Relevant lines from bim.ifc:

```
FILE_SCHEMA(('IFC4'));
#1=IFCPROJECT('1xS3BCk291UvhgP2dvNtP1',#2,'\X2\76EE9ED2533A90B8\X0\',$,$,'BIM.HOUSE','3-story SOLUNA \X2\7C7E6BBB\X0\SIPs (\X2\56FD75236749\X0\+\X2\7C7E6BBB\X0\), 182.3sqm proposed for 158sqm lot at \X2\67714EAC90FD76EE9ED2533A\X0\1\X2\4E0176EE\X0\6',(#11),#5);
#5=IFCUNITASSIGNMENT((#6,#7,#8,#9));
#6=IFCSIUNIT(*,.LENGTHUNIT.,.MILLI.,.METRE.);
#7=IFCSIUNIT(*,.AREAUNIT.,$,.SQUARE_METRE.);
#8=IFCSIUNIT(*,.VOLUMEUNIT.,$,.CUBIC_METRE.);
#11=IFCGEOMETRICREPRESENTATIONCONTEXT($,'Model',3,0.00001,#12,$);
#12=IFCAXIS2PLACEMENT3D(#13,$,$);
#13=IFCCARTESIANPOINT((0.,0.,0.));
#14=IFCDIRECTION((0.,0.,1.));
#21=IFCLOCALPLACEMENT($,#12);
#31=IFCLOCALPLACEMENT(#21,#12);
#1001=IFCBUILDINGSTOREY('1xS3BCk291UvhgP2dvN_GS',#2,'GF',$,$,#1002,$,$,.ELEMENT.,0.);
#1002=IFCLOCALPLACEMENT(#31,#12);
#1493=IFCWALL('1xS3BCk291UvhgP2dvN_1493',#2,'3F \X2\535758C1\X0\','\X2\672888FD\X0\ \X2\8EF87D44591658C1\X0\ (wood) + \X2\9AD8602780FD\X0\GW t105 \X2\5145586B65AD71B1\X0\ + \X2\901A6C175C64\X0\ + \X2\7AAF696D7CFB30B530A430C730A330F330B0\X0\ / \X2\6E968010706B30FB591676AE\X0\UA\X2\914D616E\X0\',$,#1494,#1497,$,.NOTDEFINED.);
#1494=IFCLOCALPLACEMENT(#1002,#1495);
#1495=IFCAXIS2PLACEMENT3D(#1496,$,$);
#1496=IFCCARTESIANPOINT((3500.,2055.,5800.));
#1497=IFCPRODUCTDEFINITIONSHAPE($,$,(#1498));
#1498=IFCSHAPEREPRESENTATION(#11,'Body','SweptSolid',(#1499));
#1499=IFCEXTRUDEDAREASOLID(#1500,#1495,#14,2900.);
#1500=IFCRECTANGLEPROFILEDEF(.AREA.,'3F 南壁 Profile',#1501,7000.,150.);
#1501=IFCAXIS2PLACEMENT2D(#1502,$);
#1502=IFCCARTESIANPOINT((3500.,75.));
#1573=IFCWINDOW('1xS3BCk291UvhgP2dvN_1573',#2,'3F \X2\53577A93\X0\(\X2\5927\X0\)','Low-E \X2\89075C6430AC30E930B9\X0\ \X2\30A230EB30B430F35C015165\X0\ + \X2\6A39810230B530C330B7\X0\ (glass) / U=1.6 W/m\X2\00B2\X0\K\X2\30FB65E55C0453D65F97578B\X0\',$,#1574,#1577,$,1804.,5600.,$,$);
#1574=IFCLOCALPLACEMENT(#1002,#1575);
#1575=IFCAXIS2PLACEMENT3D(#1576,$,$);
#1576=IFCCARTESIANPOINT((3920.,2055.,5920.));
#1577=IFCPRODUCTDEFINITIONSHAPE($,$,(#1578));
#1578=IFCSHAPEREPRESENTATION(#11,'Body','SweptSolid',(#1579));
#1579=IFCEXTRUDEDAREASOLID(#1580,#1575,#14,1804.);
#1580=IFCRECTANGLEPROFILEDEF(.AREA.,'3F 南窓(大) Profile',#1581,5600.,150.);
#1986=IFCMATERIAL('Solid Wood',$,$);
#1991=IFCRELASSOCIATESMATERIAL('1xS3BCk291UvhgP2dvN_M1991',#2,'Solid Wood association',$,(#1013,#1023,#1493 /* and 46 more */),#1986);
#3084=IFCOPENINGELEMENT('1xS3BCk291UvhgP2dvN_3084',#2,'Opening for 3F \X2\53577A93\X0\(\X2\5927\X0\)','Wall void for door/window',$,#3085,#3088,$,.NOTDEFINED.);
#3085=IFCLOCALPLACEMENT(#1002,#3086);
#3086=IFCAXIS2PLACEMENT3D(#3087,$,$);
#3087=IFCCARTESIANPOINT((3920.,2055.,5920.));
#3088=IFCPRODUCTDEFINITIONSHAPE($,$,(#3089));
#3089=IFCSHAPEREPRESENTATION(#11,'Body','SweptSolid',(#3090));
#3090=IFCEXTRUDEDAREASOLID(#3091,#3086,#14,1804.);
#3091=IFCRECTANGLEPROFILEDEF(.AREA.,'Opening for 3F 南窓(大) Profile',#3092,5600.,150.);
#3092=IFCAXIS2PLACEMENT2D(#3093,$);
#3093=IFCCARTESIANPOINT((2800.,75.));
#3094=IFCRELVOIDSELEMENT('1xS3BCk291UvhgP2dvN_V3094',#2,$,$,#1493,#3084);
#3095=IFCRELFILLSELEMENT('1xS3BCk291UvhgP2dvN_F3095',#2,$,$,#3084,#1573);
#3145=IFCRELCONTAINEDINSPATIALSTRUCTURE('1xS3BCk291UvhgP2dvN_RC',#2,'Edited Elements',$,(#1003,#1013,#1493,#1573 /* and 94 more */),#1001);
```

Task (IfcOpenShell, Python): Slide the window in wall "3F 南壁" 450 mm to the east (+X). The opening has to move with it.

```python
import ifcopenshell
import ifcopenshell.api.geometry
import ifcopenshell.util.placement

model = ifcopenshell.open("bim.ifc")

window = model.by_guid("1xS3BCk291UvhgP2dvN_1573")
opening = window.FillsVoids[0].RelatingOpeningElement
wall = opening.VoidsElements[0].RelatingBuildingElement

wall_matrix = ifcopenshell.util.placement.get_local_placement(wall.ObjectPlacement)
shift = wall_matrix[:3, 0] * 450.0
before = ifcopenshell.util.placement.get_local_placement(window.ObjectPlacement)[:3, 3].copy()

# The window is not placed relative to its opening, so move both.
for product in (opening, window):
    matrix = ifcopenshell.util.placement.get_local_placement(product.ObjectPlacement)
    matrix[:3, 3] += shift
    ifcopenshell.api.geometry.edit_object_placement(model, product=product, matrix=matrix, is_si=False)

after = ifcopenshell.util.placement.get_local_placement(window.ObjectPlacement)[:3, 3]
print("window moved by", (after - before).round(3) + 0.0)

model.write("bim-out.ifc")
```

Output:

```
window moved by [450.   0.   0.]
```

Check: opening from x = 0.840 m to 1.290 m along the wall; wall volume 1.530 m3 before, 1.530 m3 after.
